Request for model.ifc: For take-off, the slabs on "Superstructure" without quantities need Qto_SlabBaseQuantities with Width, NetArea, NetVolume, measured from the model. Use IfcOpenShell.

First a look at what the model holds.

```python
import ifcopenshell
import ifcopenshell.util.element
import ifcopenshell.util.unit

model = ifcopenshell.open("model.ifc")
print(model.schema)
for unit_type in ("LENGTHUNIT", "AREAUNIT", "VOLUMEUNIT"):
    print(unit_type, ifcopenshell.util.unit.calculate_unit_scale(model, unit_type))
storey = next(s for s in model.by_type("IfcBuildingStorey") if s.Name == "Superstructure")
slabs = [e for e in ifcopenshell.util.element.get_decomposition(storey) if e.is_a("IfcSlab")]
for e in sorted(slabs, key=lambda e: e.id()):
    print(e.id(), e.is_a(), e.Name, list(ifcopenshell.util.element.get_psets(e, qtos_only=True)), sep=" | ")
```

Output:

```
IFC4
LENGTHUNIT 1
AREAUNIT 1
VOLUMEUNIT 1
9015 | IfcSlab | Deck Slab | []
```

```python
import ifcopenshell
import ifcopenshell.api.pset
import ifcopenshell.geom
import ifcopenshell.util.element
import ifcopenshell.util.shape
import ifcopenshell.util.unit

model = ifcopenshell.open("model.ifc")
unit_scale = ifcopenshell.util.unit.calculate_unit_scale(model)
area_scale = ifcopenshell.util.unit.calculate_unit_scale(model, "AREAUNIT")
volume_scale = ifcopenshell.util.unit.calculate_unit_scale(model, "VOLUMEUNIT")
settings = ifcopenshell.geom.settings()

storey = next(s for s in model.by_type("IfcBuildingStorey") if s.Name == "Superstructure")
slabs = [e for e in ifcopenshell.util.element.get_decomposition(storey) if e.is_a("IfcSlab")]

for e in sorted(slabs, key=lambda e: e.id()):
    if ifcopenshell.util.element.get_psets(e, qtos_only=True, should_inherit=False):
        continue
    # Geometry comes back in metres, in the element's own axes.
    shape = ifcopenshell.geom.create_shape(settings, e)
    values = {
        "Width": ifcopenshell.util.shape.get_z(shape.geometry) / unit_scale,
        "NetArea": ifcopenshell.util.shape.get_footprint_area(shape.geometry) / area_scale,
        "NetVolume": ifcopenshell.util.shape.get_volume(shape.geometry) / volume_scale,
    }
    qto = ifcopenshell.api.pset.add_qto(model, product=e, name="Qto_SlabBaseQuantities")
    ifcopenshell.api.pset.edit_qto(model, qto=qto, properties=values)
    print(e.id(), {k: round(v, 3) for k, v in values.items()})

model.write("model_rev.ifc")
```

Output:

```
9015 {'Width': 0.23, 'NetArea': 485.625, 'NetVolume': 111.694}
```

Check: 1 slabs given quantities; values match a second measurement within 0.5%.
